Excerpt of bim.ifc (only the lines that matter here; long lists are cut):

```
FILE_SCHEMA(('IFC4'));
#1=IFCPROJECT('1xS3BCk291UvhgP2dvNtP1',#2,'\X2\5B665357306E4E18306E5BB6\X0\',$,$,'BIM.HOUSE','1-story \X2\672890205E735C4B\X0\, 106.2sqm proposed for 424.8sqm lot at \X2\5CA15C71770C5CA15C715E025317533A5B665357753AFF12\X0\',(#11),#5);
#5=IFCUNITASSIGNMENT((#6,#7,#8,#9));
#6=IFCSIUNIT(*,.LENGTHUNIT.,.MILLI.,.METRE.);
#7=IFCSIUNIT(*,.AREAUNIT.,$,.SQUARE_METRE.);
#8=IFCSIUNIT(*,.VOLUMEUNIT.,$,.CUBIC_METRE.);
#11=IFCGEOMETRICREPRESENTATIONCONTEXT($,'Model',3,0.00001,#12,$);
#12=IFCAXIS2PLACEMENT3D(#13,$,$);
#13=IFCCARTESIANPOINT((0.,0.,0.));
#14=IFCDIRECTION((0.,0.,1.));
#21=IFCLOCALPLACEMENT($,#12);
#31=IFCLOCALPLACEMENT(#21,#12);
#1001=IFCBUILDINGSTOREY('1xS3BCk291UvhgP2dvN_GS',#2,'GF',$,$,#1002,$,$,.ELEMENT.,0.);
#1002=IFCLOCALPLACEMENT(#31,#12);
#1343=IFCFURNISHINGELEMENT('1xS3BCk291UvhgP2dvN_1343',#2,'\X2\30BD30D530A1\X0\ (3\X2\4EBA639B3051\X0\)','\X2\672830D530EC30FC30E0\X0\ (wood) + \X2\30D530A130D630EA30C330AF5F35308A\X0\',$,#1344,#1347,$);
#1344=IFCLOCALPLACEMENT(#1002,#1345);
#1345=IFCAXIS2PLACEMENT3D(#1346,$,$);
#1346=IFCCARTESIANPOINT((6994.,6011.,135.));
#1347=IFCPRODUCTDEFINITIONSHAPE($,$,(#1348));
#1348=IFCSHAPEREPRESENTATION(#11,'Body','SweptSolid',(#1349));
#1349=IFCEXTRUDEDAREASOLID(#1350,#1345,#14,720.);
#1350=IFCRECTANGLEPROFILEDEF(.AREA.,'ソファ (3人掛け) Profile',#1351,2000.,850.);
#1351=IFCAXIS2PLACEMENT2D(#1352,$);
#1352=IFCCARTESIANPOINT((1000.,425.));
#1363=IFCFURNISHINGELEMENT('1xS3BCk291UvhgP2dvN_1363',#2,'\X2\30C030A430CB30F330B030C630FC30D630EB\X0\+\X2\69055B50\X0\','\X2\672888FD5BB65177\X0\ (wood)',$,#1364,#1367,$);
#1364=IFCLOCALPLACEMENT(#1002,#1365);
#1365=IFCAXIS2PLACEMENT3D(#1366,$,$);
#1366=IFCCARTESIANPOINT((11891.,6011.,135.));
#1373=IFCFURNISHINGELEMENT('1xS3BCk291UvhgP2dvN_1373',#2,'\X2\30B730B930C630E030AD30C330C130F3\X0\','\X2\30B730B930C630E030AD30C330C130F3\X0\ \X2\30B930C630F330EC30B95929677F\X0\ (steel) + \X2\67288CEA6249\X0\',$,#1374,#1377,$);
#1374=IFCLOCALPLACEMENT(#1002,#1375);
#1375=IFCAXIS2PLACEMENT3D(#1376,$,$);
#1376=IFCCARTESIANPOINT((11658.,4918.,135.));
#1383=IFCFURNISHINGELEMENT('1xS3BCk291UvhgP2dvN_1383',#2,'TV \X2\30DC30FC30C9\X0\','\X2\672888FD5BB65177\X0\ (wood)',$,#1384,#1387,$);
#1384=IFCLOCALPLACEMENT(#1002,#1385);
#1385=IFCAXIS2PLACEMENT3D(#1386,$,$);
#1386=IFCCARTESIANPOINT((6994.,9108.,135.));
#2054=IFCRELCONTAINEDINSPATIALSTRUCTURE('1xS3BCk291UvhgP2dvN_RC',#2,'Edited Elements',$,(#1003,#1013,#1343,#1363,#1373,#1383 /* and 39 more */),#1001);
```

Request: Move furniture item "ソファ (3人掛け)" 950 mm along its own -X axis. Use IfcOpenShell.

```python
import ifcopenshell
import ifcopenshell.api.geometry
import ifcopenshell.util.placement
import ifcopenshell.util.unit

model = ifcopenshell.open("bim.ifc")
unit_scale = ifcopenshell.util.unit.calculate_unit_scale(model)

item = model.by_guid("1xS3BCk291UvhgP2dvN_1343")
matrix = ifcopenshell.util.placement.get_local_placement(item.ObjectPlacement)
matrix[:3, 3] -= matrix[:3, 0] * 0.95 / unit_scale
ifcopenshell.api.geometry.edit_object_placement(model, product=item, matrix=matrix, is_si=False)

print(ifcopenshell.util.placement.get_local_placement(item.ObjectPlacement).round(3) + 0.0)

model.write("bim_updated.ifc")
```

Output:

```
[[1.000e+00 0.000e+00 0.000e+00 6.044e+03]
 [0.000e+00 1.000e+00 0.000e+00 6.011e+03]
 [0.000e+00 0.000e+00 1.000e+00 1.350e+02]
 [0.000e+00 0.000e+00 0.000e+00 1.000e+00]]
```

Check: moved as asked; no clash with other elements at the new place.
